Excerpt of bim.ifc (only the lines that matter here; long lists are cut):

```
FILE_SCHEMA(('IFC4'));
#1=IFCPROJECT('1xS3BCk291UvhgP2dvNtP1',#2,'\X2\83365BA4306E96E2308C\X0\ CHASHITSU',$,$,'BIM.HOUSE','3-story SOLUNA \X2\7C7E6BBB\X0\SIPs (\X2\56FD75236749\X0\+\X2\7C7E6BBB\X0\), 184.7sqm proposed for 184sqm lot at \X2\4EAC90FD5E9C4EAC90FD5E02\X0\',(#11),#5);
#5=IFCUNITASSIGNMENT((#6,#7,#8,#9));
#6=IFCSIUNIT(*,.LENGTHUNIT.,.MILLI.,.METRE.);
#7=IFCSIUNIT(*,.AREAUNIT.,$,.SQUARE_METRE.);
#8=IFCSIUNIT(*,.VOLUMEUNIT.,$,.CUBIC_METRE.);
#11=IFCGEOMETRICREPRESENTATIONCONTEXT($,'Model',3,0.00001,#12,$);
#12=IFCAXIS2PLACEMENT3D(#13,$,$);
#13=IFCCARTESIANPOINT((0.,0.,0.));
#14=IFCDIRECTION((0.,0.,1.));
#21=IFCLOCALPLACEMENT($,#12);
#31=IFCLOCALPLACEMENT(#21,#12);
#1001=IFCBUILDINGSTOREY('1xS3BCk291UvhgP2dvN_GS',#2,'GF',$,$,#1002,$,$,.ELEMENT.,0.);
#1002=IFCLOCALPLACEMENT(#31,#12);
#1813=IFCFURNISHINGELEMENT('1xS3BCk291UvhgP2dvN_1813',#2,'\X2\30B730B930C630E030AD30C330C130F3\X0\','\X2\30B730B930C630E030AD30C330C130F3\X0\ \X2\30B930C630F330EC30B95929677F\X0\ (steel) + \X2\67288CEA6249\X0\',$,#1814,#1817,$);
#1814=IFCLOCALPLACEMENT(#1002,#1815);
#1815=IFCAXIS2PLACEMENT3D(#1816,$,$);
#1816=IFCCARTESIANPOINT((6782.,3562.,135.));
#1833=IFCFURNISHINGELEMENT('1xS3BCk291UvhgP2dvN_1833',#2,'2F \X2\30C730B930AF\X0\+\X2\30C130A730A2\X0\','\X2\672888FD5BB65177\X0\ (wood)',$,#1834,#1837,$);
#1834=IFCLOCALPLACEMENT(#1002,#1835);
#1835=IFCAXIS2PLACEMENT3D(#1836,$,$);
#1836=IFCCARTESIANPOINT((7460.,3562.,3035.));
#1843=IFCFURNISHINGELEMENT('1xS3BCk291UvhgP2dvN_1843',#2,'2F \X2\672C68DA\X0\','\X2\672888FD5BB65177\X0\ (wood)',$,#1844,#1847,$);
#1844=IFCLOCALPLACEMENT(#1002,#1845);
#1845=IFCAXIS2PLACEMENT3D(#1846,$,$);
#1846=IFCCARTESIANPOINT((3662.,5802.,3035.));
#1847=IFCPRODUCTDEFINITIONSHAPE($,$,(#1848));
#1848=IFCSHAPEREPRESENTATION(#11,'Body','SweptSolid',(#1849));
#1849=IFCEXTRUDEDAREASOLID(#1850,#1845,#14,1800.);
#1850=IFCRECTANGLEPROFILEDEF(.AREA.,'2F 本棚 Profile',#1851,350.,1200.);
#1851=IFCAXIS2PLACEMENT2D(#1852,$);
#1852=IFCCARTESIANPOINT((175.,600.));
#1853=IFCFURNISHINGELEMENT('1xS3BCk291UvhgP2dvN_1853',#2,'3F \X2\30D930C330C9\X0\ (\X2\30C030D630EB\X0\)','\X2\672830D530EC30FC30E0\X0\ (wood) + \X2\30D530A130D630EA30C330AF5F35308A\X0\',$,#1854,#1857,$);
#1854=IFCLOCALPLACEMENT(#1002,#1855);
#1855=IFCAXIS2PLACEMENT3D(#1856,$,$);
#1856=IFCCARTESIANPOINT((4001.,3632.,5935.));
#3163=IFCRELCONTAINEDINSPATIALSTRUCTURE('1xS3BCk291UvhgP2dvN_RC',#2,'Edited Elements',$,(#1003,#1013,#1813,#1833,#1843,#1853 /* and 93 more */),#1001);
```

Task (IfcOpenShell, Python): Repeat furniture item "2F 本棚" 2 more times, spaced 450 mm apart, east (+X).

```python
import numpy as np
import ifcopenshell
import ifcopenshell.api.geometry
import ifcopenshell.api.root
import ifcopenshell.util.element
import ifcopenshell.util.placement

model = ifcopenshell.open("bim.ifc")


def reuse_history(source, copy):
    """copy_class also copies each property set's owner history, people and application; keep the originals."""
    for rel in copy.IsDefinedBy:
        if rel.is_a("IfcRelDefinesByProperties") and (history := rel.RelatingPropertyDefinition.OwnerHistory):
            rel.RelatingPropertyDefinition.OwnerHistory = source.OwnerHistory
            ifcopenshell.util.element.remove_deep2(model, history)


source = model.by_id(1843)
base = ifcopenshell.util.placement.get_local_placement(source.ObjectPlacement)
step = np.array([1.0, 0.0, 0.0]) * 450.0

for i in range(1, 3):
    copy = ifcopenshell.api.root.copy_class(model, product=source)
    copy.Representation = ifcopenshell.util.element.copy_deep(
        model, source.Representation, exclude=["IfcGeometricRepresentationContext", "IfcRepresentationMap"]
    )
    reuse_history(source, copy)
    matrix = base.copy()
    matrix[:3, 3] += i * step
    print("added at", matrix[:3, 3].round(3) + 0.0)
    ifcopenshell.api.geometry.edit_object_placement(model, product=copy, matrix=matrix, is_si=False)

model.write("bim-out.ifc")
```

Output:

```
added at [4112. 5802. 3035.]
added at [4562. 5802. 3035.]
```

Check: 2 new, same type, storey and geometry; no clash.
